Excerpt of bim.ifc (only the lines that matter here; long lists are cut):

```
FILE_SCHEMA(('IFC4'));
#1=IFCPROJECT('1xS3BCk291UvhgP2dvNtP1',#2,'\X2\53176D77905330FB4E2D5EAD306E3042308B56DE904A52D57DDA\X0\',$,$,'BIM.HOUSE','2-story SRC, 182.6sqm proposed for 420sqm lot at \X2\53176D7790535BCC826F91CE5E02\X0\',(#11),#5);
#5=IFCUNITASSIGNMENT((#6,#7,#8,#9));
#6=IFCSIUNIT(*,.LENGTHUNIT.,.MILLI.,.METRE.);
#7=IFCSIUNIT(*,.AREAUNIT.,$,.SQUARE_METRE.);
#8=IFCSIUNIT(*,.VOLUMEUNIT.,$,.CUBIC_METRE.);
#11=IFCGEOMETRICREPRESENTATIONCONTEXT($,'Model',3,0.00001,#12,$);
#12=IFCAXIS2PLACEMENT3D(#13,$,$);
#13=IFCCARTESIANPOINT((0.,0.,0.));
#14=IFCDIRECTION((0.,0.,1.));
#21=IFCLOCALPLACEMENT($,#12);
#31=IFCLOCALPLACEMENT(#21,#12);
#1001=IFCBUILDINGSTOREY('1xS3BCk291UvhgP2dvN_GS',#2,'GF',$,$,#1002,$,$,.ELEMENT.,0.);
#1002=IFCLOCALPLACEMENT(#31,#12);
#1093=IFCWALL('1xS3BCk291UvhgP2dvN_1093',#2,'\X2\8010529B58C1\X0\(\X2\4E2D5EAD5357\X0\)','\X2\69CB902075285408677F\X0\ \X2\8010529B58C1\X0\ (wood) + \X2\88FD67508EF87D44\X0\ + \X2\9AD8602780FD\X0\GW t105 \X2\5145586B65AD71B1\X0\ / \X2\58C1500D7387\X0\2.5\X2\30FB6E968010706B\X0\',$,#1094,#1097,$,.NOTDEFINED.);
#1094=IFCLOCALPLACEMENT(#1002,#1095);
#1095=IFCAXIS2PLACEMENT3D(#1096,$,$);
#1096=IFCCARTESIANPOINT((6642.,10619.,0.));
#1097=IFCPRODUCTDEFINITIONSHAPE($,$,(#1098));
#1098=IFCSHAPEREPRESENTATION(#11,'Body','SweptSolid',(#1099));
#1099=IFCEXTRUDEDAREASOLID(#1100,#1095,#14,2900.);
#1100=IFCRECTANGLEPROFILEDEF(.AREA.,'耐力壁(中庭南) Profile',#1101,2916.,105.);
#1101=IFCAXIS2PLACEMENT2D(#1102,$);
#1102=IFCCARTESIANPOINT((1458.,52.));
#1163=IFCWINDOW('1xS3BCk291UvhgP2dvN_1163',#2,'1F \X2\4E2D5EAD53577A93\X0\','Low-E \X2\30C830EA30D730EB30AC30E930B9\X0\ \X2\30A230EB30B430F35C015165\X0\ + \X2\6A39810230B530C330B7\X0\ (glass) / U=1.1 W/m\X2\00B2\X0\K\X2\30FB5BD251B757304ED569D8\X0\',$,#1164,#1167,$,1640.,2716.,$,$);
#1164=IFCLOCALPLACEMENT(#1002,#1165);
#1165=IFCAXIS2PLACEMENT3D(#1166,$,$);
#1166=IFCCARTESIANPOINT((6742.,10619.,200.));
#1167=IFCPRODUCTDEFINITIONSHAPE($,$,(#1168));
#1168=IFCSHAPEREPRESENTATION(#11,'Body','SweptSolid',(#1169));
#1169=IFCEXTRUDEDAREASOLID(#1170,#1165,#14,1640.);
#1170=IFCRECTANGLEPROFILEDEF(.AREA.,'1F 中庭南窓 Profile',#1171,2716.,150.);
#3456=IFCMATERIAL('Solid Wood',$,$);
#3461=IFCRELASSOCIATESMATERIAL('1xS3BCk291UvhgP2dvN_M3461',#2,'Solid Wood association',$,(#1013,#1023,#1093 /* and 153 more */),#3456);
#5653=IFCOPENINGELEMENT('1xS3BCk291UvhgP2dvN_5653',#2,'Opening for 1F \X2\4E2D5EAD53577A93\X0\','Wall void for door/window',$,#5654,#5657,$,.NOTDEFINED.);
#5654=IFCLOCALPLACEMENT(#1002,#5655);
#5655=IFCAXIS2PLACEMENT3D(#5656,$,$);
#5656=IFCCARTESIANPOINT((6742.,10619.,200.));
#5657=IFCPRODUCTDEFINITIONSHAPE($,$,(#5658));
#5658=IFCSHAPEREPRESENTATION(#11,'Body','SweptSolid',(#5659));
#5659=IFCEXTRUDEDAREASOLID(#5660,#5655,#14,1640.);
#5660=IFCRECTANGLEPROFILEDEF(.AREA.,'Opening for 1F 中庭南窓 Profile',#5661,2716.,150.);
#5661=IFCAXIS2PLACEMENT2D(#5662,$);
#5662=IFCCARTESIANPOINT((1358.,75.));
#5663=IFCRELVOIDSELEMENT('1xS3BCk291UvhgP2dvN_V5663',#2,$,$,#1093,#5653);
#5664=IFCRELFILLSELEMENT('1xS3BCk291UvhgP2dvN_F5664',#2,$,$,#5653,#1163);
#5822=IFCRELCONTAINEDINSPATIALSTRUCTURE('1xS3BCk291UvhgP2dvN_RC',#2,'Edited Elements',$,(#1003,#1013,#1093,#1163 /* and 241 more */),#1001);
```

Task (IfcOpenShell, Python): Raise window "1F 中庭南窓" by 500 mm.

```python
import numpy as np
import ifcopenshell
import ifcopenshell.api.geometry
import ifcopenshell.util.placement
import ifcopenshell.util.unit

model = ifcopenshell.open("bim.ifc")
unit_scale = ifcopenshell.util.unit.calculate_unit_scale(model)

window = model.by_id(1163)
opening = window.FillsVoids[0].RelatingOpeningElement
dz = 0.5 / unit_scale

shift = np.array([0.0, 0.0, dz])
# The window is not placed relative to its opening, so move both.
for product in (opening, window):
    matrix = ifcopenshell.util.placement.get_local_placement(product.ObjectPlacement)
    matrix[:3, 3] += shift
    ifcopenshell.api.geometry.edit_object_placement(model, product=product, matrix=matrix, is_si=False)

print(f"moved by {dz * unit_scale:+.3f} m")

model.write("bim_rev.ifc")
```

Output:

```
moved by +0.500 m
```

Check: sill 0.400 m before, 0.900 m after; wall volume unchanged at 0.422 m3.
